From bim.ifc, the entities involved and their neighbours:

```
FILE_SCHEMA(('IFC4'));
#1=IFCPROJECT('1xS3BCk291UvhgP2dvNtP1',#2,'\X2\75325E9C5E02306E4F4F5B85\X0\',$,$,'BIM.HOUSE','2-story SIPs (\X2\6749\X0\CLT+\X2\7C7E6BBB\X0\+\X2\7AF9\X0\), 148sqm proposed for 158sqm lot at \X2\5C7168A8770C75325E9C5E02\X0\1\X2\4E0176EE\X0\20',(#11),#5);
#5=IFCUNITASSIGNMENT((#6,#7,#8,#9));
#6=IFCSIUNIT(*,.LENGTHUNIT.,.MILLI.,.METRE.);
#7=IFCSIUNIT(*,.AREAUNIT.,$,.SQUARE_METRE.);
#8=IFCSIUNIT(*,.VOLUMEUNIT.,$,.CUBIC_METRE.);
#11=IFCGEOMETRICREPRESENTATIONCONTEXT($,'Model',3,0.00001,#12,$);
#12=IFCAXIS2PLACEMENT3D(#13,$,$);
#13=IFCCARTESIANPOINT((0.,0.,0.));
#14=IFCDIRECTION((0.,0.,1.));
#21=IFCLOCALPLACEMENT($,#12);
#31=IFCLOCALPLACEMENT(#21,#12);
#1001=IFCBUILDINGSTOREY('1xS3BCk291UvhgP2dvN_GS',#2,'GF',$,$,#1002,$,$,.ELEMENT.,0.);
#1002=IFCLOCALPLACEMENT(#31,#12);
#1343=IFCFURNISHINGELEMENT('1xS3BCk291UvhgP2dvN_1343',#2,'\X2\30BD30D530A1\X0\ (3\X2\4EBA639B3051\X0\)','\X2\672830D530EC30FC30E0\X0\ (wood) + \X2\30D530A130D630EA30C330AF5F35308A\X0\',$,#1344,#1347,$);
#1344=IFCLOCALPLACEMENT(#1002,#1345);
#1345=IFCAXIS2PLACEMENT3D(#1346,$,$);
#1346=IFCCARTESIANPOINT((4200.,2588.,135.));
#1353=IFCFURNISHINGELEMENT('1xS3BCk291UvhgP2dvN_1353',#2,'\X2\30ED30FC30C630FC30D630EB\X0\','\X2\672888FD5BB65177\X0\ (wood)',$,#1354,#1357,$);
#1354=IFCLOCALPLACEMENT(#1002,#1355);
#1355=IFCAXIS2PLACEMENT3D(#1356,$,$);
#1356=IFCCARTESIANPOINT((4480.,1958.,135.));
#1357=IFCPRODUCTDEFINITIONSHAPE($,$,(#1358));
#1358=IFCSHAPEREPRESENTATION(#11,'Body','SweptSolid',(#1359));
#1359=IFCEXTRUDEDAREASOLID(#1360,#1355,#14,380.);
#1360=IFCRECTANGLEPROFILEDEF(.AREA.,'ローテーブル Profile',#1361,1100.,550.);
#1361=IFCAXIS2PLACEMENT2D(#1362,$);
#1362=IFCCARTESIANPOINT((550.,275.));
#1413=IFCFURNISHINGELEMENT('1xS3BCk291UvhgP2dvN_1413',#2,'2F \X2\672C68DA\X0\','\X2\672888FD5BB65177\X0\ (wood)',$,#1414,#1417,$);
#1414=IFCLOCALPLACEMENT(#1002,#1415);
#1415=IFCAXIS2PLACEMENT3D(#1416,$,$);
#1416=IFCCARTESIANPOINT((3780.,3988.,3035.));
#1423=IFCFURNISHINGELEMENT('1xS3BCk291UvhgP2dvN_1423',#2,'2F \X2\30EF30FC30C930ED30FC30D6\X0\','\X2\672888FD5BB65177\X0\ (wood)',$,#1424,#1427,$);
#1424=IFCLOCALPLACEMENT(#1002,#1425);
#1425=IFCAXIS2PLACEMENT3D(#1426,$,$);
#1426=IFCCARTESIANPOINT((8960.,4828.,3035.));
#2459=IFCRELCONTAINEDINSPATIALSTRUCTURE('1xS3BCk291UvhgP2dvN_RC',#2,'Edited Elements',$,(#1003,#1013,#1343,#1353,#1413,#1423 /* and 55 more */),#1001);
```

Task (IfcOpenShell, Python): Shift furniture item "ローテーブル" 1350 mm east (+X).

```python
import ifcopenshell
import ifcopenshell.api.geometry
import ifcopenshell.util.placement
import ifcopenshell.util.unit

model = ifcopenshell.open("bim.ifc")
unit_scale = ifcopenshell.util.unit.calculate_unit_scale(model)

item = model.by_guid("1xS3BCk291UvhgP2dvN_1353")
matrix = ifcopenshell.util.placement.get_local_placement(item.ObjectPlacement)
matrix[0, 3] += 1.35 / unit_scale
ifcopenshell.api.geometry.edit_object_placement(model, product=item, matrix=matrix, is_si=False)

print(ifcopenshell.util.placement.get_local_placement(item.ObjectPlacement).round(3) + 0.0)

model.write("bim_edited.ifc")
```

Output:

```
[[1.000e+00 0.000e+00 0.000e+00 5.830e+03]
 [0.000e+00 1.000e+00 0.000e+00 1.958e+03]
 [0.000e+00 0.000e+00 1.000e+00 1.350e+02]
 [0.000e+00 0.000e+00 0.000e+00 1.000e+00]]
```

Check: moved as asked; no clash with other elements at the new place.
